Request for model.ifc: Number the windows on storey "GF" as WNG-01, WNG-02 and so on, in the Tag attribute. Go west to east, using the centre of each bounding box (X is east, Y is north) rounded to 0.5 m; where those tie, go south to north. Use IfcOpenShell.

First a look at what the model holds.

```python
import ifcopenshell
import ifcopenshell.util.element
import ifcopenshell.util.placement

model = ifcopenshell.open("model.ifc")
print(model.schema)
storey = next(s for s in model.by_type("IfcBuildingStorey") if s.Name == "GF")
windows = [e for e in ifcopenshell.util.element.get_decomposition(storey) if e.is_a("IfcWindow")]
for e in sorted(windows, key=lambda e: e.id()):
    origin = ifcopenshell.util.placement.get_local_placement(e.ObjectPlacement)[:3, 3]
    print(e.id(), e.Tag, e.Name, origin.round(2) + 0.0, sep=" | ")
```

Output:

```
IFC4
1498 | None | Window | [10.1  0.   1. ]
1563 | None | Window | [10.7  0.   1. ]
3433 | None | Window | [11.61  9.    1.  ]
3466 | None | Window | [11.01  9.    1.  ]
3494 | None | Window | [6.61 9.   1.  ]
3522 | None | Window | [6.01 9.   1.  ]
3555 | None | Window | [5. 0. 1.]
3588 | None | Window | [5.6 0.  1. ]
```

```python
import ifcopenshell
import ifcopenshell.geom
import ifcopenshell.util.element
import ifcopenshell.util.shape

model = ifcopenshell.open("model.ifc")
settings = ifcopenshell.geom.settings()
settings.set("use-world-coords", True)


def centre(element):
    shape = ifcopenshell.geom.create_shape(settings, element)
    return ifcopenshell.util.shape.get_bbox_centroid(shape.geometry)


storey = next(s for s in model.by_type("IfcBuildingStorey") if s.Name == "GF")
windows = [e for e in ifcopenshell.util.element.get_decomposition(storey) if e.is_a("IfcWindow")]

# Insertion points can sit at a corner or the storey origin, so sort by the geometry (in metres).
centres = {e: centre(e) for e in windows}
windows.sort(key=lambda e: (round(centres[e][0] / 0.5), centres[e][1]))

for i, e in enumerate(windows, start=1):
    number = f"WNG-{i:02d}"
    e.Tag = number
    print(e.id(), number)

model.write("model-out.ifc")
```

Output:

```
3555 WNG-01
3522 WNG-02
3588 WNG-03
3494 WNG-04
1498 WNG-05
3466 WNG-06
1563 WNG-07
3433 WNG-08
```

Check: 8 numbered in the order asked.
